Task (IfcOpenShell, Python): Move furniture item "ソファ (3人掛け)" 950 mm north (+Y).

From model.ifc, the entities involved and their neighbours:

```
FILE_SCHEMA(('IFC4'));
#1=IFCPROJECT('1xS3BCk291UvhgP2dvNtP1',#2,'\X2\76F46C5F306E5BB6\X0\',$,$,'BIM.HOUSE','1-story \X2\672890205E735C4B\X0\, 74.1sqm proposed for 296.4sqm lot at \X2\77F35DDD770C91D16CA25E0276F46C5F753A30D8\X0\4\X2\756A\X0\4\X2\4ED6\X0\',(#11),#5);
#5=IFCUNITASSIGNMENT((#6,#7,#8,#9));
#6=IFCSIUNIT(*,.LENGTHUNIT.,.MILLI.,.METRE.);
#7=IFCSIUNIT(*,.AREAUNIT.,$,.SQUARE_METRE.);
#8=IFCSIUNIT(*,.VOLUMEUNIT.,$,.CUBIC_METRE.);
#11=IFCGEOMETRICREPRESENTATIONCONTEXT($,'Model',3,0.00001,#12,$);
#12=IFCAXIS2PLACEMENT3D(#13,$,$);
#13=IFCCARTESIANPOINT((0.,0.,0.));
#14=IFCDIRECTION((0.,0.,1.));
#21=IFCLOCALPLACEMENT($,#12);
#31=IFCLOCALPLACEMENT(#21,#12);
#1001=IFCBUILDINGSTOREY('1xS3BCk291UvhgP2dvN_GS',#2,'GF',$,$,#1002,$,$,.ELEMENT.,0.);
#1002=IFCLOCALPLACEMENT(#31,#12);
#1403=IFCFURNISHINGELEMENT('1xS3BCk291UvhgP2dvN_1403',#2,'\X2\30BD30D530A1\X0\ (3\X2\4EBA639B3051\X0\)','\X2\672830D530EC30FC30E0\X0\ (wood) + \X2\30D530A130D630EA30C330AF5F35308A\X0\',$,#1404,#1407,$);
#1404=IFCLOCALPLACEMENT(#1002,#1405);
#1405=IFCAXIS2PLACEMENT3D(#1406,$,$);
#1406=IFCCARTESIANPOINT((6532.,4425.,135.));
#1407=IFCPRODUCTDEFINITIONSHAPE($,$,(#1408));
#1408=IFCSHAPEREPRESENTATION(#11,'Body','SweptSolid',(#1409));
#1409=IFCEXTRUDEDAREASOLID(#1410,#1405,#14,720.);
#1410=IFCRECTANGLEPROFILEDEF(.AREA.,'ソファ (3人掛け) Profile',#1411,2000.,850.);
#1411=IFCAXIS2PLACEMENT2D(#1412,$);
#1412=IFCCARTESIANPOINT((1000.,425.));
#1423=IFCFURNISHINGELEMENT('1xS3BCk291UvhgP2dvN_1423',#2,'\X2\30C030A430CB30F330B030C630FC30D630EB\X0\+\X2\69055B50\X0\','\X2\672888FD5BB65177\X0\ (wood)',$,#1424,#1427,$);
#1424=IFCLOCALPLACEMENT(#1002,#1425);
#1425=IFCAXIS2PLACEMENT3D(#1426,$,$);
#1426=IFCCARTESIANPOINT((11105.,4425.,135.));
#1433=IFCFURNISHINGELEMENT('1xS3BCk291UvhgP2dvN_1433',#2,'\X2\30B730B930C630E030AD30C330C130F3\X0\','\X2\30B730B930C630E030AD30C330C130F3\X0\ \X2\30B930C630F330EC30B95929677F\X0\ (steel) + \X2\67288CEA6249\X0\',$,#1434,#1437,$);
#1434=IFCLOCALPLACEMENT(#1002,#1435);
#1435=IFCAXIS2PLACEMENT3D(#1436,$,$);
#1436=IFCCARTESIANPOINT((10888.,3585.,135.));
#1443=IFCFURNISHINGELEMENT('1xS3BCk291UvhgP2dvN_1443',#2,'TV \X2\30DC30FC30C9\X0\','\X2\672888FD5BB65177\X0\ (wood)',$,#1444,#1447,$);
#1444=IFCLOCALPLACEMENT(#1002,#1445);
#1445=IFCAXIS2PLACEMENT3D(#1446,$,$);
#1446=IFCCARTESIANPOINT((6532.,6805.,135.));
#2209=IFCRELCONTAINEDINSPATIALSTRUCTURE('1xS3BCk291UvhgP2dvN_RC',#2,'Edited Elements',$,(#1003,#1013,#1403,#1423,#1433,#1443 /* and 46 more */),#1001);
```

```python
import ifcopenshell
import ifcopenshell.api.geometry
import ifcopenshell.util.placement

model = ifcopenshell.open("model.ifc")

item = model.by_guid("1xS3BCk291UvhgP2dvN_1403")
matrix = ifcopenshell.util.placement.get_local_placement(item.ObjectPlacement)
matrix[1, 3] += 950.0
ifcopenshell.api.geometry.edit_object_placement(model, product=item, matrix=matrix, is_si=False)

print(ifcopenshell.util.placement.get_local_placement(item.ObjectPlacement).round(3) + 0.0)

model.write("model_rev.ifc")
```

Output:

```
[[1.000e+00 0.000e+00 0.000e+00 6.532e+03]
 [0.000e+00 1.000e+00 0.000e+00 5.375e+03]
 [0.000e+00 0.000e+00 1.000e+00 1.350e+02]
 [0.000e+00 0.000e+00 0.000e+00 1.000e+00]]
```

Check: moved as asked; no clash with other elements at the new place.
